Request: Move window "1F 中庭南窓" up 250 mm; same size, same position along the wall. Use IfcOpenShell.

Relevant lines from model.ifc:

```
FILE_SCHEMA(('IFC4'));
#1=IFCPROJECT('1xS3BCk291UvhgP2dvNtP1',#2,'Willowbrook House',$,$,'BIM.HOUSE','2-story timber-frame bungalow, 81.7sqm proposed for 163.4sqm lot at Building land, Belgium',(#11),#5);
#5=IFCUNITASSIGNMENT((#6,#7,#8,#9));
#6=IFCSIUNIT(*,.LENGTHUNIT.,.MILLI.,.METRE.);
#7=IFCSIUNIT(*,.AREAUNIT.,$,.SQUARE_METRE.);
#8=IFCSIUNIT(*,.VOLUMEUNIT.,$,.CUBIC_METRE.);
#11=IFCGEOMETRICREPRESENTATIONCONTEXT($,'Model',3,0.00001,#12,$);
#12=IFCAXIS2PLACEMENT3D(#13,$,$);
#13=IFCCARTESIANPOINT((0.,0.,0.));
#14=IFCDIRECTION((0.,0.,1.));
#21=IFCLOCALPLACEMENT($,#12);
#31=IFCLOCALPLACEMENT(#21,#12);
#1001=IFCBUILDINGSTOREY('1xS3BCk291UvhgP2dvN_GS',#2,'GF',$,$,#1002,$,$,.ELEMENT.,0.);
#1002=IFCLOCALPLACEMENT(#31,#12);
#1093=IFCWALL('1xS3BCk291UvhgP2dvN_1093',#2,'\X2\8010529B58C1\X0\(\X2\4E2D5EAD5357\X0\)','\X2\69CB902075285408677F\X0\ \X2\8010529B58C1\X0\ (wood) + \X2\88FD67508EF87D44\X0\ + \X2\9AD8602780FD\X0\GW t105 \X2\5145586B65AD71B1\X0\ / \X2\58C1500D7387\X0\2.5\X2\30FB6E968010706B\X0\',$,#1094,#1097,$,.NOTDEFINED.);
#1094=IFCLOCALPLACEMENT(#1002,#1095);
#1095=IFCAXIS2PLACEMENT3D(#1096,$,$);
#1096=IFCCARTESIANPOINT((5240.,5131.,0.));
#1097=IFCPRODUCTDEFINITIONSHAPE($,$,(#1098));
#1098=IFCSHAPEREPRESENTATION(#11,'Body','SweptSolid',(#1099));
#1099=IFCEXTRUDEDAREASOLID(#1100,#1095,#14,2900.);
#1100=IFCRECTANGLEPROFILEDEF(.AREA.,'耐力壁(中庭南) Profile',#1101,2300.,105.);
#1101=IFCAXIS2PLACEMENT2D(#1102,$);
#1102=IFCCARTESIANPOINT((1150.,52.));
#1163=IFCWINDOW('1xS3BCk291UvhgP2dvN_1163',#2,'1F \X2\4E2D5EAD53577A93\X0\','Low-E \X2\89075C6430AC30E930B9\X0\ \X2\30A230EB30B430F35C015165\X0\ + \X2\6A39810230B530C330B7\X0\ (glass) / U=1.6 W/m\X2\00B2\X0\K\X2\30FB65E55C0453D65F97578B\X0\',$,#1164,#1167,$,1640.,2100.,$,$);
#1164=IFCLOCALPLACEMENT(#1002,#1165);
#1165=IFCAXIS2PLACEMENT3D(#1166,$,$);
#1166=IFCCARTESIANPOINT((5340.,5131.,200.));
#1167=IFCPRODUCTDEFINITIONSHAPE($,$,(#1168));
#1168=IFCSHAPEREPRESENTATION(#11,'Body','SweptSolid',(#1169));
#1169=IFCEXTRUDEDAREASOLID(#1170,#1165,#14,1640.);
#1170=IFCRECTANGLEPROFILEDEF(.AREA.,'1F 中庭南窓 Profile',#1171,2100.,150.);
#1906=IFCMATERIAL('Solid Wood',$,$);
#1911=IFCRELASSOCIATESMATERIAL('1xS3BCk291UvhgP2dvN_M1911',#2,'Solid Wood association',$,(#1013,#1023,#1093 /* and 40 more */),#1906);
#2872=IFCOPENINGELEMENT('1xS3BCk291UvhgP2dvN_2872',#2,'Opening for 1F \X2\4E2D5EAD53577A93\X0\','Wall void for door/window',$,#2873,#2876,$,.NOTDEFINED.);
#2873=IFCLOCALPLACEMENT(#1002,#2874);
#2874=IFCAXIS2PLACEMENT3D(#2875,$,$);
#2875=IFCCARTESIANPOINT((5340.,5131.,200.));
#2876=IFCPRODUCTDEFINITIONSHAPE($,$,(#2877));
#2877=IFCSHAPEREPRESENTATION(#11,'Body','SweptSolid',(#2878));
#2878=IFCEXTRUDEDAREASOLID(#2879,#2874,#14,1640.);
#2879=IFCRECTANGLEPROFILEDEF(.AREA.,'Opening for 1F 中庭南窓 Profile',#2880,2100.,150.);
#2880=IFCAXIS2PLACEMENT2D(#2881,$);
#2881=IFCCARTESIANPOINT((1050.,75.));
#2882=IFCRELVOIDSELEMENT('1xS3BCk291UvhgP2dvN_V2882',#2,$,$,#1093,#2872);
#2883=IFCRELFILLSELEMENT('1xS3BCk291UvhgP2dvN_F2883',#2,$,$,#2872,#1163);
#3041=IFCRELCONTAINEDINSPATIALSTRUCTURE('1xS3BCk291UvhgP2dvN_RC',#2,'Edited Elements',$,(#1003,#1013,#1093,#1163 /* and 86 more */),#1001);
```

```python
import numpy as np
import ifcopenshell
import ifcopenshell.api.geometry
import ifcopenshell.util.placement
import ifcopenshell.util.unit

model = ifcopenshell.open("model.ifc")
unit_scale = ifcopenshell.util.unit.calculate_unit_scale(model)

window = model.by_id(1163)
opening = window.FillsVoids[0].RelatingOpeningElement
dz = 250.0

shift = np.array([0.0, 0.0, dz])
# The window is not placed relative to its opening, so move both.
for product in (opening, window):
    matrix = ifcopenshell.util.placement.get_local_placement(product.ObjectPlacement)
    matrix[:3, 3] += shift
    ifcopenshell.api.geometry.edit_object_placement(model, product=product, matrix=matrix, is_si=False)

print(f"moved by {dz * unit_scale:+.3f} m")

model.write("model_v2.ifc")
```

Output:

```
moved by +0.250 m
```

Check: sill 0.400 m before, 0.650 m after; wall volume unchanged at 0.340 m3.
